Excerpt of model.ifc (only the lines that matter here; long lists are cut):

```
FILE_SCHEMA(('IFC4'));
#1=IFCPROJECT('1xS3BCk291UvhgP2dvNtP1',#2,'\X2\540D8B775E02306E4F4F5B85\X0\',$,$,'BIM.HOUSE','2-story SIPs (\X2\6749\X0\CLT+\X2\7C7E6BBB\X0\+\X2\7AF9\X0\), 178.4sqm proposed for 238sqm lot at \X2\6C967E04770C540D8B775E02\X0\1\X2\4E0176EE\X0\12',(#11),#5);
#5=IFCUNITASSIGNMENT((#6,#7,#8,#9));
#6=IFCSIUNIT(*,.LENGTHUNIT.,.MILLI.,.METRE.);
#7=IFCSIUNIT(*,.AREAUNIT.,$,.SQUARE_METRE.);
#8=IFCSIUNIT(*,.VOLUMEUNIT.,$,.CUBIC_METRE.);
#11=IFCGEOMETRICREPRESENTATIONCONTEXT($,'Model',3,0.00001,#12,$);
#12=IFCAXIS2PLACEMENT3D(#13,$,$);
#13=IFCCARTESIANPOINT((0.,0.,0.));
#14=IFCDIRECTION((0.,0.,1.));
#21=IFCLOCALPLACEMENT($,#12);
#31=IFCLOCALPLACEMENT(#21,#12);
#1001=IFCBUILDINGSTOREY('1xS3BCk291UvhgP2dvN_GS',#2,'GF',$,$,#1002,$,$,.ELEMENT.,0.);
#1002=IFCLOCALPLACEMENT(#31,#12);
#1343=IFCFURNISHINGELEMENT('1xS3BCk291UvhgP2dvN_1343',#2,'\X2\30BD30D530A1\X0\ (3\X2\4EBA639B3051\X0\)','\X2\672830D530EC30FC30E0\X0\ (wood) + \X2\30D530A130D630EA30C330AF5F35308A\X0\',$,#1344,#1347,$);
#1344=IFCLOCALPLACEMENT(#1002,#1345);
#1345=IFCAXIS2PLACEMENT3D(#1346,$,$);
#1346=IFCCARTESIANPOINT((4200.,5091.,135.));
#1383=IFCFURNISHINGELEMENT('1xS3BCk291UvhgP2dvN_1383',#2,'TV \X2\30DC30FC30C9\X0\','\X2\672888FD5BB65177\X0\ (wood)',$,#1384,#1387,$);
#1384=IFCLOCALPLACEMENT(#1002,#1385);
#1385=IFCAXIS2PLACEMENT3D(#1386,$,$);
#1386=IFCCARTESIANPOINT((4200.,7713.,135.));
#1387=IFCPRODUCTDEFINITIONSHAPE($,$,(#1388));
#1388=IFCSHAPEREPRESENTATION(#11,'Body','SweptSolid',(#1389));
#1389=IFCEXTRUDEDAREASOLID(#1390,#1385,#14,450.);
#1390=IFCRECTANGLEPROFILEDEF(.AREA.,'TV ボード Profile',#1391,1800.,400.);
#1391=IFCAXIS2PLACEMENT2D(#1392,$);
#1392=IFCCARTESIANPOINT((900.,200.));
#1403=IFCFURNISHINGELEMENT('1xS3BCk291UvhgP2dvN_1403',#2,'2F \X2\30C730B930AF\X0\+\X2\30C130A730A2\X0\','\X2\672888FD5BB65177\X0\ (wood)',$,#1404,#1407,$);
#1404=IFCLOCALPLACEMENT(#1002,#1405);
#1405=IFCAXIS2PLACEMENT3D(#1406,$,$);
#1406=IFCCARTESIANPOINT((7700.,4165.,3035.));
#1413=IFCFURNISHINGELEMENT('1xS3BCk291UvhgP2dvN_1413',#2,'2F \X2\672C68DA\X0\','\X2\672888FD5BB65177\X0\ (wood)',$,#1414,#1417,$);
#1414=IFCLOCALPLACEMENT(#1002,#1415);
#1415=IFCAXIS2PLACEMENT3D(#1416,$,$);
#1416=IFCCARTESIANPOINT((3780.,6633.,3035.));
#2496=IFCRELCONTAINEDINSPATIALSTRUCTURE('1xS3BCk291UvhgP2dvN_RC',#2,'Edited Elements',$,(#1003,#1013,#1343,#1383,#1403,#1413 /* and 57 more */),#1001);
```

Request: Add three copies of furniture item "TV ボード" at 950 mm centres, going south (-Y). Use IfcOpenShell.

```python
import numpy as np
import ifcopenshell
import ifcopenshell.api.geometry
import ifcopenshell.api.root
import ifcopenshell.util.element
import ifcopenshell.util.placement
import ifcopenshell.util.unit

model = ifcopenshell.open("model.ifc")
unit_scale = ifcopenshell.util.unit.calculate_unit_scale(model)


def reuse_history(source, copy):
    """copy_class also copies each property set's owner history, people and application; keep the originals."""
    for rel in copy.IsDefinedBy:
        if rel.is_a("IfcRelDefinesByProperties") and (history := rel.RelatingPropertyDefinition.OwnerHistory):
            rel.RelatingPropertyDefinition.OwnerHistory = source.OwnerHistory
            ifcopenshell.util.element.remove_deep2(model, history)


source = model.by_guid("1xS3BCk291UvhgP2dvN_1383")
base = ifcopenshell.util.placement.get_local_placement(source.ObjectPlacement)
step = np.array([0.0, -1.0, 0.0]) * 0.95 / unit_scale

for i in range(1, 4):
    copy = ifcopenshell.api.root.copy_class(model, product=source)
    copy.Representation = ifcopenshell.util.element.copy_deep(
        model, source.Representation, exclude=["IfcGeometricRepresentationContext", "IfcRepresentationMap"]
    )
    reuse_history(source, copy)
    matrix = base.copy()
    matrix[:3, 3] += i * step
    print("added at", matrix[:3, 3].round(3) + 0.0)
    ifcopenshell.api.geometry.edit_object_placement(model, product=copy, matrix=matrix, is_si=False)

model.write("model_v2.ifc")
```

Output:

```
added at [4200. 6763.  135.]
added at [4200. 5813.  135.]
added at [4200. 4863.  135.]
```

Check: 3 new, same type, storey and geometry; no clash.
